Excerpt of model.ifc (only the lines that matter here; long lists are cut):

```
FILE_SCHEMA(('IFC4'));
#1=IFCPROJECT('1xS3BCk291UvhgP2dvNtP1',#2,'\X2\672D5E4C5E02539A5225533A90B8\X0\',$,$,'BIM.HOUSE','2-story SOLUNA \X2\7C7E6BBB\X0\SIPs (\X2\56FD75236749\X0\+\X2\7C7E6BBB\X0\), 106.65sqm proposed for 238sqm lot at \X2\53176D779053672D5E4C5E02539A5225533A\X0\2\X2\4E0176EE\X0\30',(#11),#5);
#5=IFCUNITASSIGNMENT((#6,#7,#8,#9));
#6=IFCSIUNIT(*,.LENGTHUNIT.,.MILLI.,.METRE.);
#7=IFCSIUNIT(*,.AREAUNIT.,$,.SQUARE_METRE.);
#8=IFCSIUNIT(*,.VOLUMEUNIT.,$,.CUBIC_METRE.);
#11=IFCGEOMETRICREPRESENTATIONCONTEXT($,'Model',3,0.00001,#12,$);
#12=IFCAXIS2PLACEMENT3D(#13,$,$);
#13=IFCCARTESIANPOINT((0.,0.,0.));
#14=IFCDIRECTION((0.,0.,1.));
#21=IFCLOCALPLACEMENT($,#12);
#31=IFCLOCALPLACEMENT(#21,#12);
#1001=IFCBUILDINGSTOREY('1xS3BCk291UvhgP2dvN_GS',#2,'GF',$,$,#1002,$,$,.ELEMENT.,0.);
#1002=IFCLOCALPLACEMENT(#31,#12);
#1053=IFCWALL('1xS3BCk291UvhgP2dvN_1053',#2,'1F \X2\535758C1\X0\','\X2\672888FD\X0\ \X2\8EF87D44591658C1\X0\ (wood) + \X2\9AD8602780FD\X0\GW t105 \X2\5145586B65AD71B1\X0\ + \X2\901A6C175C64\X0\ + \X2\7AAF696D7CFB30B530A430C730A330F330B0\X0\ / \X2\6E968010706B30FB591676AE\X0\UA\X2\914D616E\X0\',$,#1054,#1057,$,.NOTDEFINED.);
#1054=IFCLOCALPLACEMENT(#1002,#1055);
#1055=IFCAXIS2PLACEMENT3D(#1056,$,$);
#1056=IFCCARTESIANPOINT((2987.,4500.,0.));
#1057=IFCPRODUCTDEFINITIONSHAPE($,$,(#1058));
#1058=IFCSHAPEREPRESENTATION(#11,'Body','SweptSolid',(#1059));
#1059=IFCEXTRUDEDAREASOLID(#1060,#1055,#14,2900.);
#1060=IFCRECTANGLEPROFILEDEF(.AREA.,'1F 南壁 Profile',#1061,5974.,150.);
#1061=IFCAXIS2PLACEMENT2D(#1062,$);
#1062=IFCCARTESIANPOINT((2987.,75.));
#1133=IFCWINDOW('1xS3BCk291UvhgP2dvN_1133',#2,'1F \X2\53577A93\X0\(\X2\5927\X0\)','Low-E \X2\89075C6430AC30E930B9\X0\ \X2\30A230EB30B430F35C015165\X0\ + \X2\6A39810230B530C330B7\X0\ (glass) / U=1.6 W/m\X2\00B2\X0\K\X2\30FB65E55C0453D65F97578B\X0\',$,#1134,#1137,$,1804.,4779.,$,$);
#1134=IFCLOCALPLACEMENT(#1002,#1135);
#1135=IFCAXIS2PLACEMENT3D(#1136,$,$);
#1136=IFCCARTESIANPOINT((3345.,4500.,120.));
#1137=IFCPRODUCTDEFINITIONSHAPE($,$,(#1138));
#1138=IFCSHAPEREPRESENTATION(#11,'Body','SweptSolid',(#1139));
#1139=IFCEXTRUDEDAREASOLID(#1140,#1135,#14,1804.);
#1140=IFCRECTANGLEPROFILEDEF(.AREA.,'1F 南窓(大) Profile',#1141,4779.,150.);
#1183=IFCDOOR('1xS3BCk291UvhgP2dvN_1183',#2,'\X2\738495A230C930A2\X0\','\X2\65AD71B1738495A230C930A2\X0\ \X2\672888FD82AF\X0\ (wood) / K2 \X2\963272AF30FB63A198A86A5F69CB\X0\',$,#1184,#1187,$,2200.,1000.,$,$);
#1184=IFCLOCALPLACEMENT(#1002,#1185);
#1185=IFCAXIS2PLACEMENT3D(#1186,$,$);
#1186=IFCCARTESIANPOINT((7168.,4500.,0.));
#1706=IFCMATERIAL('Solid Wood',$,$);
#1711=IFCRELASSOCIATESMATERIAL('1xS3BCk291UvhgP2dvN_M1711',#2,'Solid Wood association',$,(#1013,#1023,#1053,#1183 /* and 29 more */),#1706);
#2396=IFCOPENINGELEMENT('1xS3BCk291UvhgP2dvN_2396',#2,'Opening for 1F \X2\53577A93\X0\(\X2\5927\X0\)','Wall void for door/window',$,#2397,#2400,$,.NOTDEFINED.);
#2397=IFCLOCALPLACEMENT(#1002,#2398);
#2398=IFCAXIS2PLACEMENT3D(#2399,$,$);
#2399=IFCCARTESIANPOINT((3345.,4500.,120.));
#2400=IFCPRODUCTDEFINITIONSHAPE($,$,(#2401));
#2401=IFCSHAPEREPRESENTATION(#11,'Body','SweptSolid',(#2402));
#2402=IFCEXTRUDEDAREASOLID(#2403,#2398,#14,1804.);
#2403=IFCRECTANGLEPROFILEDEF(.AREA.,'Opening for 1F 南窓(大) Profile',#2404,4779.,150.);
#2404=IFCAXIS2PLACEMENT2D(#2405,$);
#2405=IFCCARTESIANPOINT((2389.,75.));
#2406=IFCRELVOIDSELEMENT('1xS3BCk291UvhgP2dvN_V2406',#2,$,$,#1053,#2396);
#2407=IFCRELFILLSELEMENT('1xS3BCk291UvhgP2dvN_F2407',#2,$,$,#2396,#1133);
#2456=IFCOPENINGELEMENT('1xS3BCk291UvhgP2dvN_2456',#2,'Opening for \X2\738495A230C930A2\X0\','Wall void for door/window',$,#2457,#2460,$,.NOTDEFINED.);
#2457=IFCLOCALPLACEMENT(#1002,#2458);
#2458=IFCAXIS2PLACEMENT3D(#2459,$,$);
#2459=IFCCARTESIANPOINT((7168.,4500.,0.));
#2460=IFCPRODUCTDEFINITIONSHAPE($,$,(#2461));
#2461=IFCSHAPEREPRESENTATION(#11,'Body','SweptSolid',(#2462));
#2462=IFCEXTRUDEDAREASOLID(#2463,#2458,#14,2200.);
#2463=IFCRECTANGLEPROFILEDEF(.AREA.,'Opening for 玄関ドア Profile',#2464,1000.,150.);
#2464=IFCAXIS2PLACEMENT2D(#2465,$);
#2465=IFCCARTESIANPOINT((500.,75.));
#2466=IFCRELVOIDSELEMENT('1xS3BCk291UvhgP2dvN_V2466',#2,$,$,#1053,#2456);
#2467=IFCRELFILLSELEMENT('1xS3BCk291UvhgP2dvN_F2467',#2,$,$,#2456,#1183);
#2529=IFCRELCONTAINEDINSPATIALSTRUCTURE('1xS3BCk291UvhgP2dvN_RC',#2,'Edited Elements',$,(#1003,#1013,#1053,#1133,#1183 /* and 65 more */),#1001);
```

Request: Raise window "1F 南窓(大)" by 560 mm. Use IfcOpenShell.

```python
import numpy as np
import ifcopenshell
import ifcopenshell.api.geometry
import ifcopenshell.util.placement
import ifcopenshell.util.unit

model = ifcopenshell.open("model.ifc")
unit_scale = ifcopenshell.util.unit.calculate_unit_scale(model)

window = model.by_id(1133)
opening = window.FillsVoids[0].RelatingOpeningElement
dz = 0.56 / unit_scale

shift = np.array([0.0, 0.0, dz])
# The window is not placed relative to its opening, so move both.
for product in (opening, window):
    matrix = ifcopenshell.util.placement.get_local_placement(product.ObjectPlacement)
    matrix[:3, 3] += shift
    ifcopenshell.api.geometry.edit_object_placement(model, product=product, matrix=matrix, is_si=False)

print(f"moved by {dz * unit_scale:+.3f} m")

model.write("model_updated.ifc")
```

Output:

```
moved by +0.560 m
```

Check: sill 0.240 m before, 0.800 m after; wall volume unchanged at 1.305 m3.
